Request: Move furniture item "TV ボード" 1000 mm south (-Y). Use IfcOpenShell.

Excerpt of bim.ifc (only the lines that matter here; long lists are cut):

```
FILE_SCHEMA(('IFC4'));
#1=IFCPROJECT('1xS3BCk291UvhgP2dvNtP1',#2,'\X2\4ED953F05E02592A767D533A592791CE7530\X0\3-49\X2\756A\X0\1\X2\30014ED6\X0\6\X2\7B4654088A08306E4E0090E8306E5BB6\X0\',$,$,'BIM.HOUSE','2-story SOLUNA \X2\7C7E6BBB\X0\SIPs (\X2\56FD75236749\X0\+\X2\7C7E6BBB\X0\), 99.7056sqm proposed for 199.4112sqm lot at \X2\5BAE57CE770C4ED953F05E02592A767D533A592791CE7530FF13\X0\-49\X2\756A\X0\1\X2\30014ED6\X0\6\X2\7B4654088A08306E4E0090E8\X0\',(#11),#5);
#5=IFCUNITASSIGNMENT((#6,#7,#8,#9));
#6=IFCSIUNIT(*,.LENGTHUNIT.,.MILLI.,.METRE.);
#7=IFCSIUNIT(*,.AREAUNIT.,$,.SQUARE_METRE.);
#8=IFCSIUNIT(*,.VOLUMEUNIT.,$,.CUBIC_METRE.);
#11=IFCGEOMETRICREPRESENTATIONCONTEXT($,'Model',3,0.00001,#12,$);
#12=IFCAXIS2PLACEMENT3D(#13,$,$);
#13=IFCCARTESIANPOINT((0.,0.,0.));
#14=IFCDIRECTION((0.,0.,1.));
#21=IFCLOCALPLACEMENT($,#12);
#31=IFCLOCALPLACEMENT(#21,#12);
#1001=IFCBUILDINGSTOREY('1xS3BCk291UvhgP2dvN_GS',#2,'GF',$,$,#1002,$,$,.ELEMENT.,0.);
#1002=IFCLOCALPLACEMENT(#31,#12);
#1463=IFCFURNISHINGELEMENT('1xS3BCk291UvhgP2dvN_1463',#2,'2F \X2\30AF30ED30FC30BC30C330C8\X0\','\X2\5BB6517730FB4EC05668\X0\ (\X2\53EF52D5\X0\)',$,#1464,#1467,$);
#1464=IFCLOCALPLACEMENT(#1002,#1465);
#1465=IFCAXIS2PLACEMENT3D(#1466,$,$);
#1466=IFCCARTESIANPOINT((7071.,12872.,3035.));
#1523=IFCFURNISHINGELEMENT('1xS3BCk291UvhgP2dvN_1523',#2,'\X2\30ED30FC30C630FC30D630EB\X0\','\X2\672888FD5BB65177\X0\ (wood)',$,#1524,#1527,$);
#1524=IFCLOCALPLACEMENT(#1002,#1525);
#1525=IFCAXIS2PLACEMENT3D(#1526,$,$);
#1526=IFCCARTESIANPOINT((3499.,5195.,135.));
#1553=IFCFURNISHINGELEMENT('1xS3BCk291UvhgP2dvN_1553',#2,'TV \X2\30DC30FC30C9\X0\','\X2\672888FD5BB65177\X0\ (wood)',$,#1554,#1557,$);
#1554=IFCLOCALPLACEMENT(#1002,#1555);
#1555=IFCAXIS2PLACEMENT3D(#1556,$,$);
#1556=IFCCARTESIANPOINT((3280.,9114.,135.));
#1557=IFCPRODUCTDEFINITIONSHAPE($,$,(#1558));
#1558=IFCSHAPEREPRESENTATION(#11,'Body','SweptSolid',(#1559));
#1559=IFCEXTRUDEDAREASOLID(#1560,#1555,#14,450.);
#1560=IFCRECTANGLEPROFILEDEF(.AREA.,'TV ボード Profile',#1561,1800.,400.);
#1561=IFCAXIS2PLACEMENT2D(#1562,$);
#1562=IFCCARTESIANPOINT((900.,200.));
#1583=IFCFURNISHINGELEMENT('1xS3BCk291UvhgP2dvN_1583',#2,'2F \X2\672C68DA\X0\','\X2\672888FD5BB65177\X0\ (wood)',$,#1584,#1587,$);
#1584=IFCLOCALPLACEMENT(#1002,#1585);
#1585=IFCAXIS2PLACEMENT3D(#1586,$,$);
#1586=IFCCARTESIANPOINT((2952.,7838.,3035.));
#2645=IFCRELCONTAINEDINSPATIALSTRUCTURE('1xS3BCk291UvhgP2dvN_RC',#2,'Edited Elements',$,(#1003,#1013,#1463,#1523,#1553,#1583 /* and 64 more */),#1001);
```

```python
import ifcopenshell
import ifcopenshell.api.geometry
import ifcopenshell.util.placement

model = ifcopenshell.open("bim.ifc")

item = model.by_guid("1xS3BCk291UvhgP2dvN_1553")
matrix = ifcopenshell.util.placement.get_local_placement(item.ObjectPlacement)
matrix[1, 3] -= 1000.0
ifcopenshell.api.geometry.edit_object_placement(model, product=item, matrix=matrix, is_si=False)

print(ifcopenshell.util.placement.get_local_placement(item.ObjectPlacement).round(3) + 0.0)

model.write("bim-out.ifc")
```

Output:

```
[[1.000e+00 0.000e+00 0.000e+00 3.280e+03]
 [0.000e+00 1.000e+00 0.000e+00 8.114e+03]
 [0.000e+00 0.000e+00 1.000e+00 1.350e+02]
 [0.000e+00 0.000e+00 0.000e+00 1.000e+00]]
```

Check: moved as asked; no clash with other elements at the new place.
